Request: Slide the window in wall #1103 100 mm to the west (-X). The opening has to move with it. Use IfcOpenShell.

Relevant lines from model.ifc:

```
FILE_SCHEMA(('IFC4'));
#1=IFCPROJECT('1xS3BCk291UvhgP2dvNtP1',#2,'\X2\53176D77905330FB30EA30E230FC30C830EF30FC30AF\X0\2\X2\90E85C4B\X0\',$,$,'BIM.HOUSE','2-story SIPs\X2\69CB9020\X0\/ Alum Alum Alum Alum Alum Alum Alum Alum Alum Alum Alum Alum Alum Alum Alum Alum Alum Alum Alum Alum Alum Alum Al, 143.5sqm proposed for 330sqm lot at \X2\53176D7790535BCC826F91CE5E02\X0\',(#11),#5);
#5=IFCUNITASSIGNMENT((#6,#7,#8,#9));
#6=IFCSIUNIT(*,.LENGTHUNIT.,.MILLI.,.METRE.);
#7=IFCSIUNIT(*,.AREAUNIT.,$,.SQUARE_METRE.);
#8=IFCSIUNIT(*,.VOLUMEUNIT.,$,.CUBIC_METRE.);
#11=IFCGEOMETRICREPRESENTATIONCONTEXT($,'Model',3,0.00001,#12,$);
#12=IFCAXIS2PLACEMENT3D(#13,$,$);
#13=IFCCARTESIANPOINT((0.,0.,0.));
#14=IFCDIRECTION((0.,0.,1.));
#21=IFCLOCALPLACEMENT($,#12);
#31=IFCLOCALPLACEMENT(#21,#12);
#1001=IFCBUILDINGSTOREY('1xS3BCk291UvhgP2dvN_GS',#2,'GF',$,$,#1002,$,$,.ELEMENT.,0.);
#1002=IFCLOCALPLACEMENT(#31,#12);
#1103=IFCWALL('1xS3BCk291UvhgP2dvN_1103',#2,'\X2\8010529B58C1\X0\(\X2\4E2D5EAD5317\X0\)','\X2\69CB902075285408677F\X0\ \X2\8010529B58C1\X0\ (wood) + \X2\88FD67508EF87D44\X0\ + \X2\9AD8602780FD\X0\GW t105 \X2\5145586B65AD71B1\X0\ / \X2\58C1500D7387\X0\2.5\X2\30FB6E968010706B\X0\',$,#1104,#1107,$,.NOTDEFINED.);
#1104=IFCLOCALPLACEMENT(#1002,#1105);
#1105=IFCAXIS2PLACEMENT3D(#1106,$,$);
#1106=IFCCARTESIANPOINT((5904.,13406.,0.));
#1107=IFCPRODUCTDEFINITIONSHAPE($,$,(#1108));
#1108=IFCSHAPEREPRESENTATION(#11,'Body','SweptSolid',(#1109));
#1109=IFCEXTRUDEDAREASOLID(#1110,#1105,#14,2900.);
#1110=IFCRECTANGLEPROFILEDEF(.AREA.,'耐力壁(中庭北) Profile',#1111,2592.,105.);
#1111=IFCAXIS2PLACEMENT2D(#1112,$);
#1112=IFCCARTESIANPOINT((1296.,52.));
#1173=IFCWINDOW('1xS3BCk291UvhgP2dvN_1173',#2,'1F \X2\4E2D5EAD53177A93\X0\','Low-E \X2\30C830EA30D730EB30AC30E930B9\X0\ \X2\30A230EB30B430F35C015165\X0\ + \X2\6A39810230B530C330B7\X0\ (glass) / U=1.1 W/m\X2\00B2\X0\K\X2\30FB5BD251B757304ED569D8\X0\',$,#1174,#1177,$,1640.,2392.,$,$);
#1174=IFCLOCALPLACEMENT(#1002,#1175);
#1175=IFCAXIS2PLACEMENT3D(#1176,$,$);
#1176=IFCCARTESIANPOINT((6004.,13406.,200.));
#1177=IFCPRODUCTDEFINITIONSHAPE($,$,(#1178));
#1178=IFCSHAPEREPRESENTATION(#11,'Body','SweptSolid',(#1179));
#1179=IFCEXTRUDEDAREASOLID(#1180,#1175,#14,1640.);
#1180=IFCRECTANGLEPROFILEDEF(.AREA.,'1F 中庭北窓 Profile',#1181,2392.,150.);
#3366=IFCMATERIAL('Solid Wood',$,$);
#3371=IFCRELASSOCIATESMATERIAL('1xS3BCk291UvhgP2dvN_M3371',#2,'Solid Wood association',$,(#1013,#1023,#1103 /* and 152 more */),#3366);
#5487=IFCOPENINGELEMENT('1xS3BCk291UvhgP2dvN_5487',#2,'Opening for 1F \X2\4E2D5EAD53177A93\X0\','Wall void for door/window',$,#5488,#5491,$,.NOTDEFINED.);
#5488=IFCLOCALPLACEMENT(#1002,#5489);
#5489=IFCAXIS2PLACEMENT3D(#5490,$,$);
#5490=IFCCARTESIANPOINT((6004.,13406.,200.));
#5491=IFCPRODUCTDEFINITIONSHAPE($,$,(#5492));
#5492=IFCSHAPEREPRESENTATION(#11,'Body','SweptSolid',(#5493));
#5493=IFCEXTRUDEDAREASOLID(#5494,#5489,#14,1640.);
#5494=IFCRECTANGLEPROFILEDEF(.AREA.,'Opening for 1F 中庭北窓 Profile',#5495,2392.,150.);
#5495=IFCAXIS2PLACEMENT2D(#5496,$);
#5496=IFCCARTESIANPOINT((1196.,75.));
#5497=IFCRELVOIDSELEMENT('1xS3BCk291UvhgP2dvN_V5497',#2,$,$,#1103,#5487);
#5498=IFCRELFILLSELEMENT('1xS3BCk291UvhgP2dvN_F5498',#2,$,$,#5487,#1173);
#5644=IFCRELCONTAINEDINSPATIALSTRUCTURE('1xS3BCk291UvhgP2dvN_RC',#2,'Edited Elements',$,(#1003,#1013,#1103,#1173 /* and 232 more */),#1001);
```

```python
import ifcopenshell
import ifcopenshell.api.geometry
import ifcopenshell.util.placement
import ifcopenshell.util.unit

model = ifcopenshell.open("model.ifc")
unit_scale = ifcopenshell.util.unit.calculate_unit_scale(model)

window = model.by_guid("1xS3BCk291UvhgP2dvN_1173")
opening = window.FillsVoids[0].RelatingOpeningElement
wall = opening.VoidsElements[0].RelatingBuildingElement

wall_matrix = ifcopenshell.util.placement.get_local_placement(wall.ObjectPlacement)
shift = wall_matrix[:3, 0] * -0.1 / unit_scale
before = ifcopenshell.util.placement.get_local_placement(window.ObjectPlacement)[:3, 3].copy()

# The window is not placed relative to its opening, so move both.
for product in (opening, window):
    matrix = ifcopenshell.util.placement.get_local_placement(product.ObjectPlacement)
    matrix[:3, 3] += shift
    ifcopenshell.api.geometry.edit_object_placement(model, product=product, matrix=matrix, is_si=False)

after = ifcopenshell.util.placement.get_local_placement(window.ObjectPlacement)[:3, 3]
print("window moved by", (after - before).round(3) + 0.0)

model.write("model_rev.ifc")
```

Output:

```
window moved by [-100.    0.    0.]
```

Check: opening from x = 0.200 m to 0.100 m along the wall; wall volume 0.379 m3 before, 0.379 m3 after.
